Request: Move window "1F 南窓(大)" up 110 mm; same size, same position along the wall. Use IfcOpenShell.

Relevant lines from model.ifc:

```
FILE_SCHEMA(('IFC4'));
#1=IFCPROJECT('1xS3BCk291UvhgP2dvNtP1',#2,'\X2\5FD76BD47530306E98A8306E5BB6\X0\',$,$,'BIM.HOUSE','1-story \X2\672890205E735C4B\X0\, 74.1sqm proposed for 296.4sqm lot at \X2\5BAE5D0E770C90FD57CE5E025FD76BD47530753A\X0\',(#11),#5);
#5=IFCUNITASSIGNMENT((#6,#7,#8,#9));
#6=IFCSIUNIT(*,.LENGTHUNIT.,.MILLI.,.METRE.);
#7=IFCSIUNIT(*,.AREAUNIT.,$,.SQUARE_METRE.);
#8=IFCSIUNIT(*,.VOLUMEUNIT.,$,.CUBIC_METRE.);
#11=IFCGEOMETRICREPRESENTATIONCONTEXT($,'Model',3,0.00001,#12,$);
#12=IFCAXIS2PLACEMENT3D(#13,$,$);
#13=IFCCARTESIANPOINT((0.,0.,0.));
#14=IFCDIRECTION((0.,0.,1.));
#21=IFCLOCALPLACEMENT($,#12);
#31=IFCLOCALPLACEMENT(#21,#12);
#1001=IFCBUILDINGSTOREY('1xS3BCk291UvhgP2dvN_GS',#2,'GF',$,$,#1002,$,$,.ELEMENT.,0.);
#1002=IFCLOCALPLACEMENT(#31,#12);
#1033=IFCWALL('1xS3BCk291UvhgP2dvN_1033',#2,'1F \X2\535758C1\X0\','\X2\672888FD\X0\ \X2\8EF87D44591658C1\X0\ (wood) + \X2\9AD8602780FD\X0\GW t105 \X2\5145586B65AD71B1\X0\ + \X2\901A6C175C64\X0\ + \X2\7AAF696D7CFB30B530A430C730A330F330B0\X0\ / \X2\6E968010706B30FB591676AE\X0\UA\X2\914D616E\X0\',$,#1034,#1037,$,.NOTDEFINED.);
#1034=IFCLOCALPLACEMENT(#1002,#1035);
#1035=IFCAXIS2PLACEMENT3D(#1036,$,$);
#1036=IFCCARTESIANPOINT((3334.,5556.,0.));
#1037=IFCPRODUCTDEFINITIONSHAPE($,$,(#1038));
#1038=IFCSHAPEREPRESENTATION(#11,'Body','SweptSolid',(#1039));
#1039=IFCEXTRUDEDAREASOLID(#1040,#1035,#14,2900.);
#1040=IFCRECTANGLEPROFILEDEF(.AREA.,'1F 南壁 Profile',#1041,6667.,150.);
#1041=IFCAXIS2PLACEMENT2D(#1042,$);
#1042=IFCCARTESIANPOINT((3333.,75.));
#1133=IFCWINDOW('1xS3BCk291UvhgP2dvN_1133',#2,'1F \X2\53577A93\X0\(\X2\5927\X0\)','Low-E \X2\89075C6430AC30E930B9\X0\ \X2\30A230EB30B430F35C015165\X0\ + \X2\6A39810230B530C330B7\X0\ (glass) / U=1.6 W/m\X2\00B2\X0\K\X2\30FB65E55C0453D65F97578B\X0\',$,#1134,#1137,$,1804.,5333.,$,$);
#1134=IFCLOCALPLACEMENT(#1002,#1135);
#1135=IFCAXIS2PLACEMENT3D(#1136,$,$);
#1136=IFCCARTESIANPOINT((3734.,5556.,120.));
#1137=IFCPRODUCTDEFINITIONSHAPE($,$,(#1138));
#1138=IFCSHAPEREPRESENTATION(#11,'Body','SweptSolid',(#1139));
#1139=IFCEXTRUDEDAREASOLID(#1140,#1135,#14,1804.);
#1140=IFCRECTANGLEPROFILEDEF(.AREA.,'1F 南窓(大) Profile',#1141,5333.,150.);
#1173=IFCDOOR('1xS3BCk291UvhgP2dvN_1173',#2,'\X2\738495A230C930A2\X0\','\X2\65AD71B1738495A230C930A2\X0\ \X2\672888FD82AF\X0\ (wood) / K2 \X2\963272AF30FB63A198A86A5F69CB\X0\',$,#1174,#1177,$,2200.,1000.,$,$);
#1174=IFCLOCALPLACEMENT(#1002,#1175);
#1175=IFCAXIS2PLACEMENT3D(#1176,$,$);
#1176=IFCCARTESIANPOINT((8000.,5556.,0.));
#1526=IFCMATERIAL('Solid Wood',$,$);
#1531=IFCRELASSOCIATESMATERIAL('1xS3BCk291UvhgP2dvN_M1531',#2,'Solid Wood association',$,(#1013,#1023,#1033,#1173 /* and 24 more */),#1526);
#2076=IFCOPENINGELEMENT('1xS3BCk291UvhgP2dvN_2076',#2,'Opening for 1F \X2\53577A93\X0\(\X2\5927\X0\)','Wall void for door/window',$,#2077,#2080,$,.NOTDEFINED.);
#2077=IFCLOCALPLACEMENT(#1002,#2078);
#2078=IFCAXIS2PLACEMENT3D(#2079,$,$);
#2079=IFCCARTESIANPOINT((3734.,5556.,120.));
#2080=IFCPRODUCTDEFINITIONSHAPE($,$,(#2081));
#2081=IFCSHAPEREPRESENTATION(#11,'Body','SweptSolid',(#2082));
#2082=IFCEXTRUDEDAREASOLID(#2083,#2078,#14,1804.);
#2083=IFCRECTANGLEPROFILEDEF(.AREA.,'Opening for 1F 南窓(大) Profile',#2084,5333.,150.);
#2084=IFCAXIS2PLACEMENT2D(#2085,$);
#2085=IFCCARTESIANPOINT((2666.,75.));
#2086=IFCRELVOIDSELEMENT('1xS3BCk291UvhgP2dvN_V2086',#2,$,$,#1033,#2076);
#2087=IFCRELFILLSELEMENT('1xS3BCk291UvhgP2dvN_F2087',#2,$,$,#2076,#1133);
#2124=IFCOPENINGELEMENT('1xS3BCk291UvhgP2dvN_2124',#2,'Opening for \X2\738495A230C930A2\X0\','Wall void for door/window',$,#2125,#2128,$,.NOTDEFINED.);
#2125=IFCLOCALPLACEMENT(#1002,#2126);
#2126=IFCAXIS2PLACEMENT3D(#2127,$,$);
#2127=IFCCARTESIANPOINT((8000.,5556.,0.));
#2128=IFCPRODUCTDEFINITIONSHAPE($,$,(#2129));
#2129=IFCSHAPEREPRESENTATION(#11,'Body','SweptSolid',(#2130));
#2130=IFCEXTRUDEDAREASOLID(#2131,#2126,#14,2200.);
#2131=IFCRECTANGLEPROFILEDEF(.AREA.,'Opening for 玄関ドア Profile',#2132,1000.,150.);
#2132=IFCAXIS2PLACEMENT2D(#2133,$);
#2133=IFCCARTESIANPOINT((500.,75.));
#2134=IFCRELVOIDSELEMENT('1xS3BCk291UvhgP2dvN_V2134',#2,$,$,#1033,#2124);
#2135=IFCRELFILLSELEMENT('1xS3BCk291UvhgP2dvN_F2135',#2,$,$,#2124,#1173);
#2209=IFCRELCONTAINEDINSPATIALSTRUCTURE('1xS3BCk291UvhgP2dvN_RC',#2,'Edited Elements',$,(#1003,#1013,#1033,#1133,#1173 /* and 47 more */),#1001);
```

```python
import numpy as np
import ifcopenshell
import ifcopenshell.api.geometry
import ifcopenshell.util.placement
import ifcopenshell.util.unit

model = ifcopenshell.open("model.ifc")
unit_scale = ifcopenshell.util.unit.calculate_unit_scale(model)

window = model.by_guid("1xS3BCk291UvhgP2dvN_1133")
opening = window.FillsVoids[0].RelatingOpeningElement
dz = 0.11 / unit_scale

shift = np.array([0.0, 0.0, dz])
# The window is not placed relative to its opening, so move both.
for product in (opening, window):
    matrix = ifcopenshell.util.placement.get_local_placement(product.ObjectPlacement)
    matrix[:3, 3] += shift
    ifcopenshell.api.geometry.edit_object_placement(model, product=product, matrix=matrix, is_si=False)

print(f"moved by {dz * unit_scale:+.3f} m")

model.write("model_edited.ifc")
```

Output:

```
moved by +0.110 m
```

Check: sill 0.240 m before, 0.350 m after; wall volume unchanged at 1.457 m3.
